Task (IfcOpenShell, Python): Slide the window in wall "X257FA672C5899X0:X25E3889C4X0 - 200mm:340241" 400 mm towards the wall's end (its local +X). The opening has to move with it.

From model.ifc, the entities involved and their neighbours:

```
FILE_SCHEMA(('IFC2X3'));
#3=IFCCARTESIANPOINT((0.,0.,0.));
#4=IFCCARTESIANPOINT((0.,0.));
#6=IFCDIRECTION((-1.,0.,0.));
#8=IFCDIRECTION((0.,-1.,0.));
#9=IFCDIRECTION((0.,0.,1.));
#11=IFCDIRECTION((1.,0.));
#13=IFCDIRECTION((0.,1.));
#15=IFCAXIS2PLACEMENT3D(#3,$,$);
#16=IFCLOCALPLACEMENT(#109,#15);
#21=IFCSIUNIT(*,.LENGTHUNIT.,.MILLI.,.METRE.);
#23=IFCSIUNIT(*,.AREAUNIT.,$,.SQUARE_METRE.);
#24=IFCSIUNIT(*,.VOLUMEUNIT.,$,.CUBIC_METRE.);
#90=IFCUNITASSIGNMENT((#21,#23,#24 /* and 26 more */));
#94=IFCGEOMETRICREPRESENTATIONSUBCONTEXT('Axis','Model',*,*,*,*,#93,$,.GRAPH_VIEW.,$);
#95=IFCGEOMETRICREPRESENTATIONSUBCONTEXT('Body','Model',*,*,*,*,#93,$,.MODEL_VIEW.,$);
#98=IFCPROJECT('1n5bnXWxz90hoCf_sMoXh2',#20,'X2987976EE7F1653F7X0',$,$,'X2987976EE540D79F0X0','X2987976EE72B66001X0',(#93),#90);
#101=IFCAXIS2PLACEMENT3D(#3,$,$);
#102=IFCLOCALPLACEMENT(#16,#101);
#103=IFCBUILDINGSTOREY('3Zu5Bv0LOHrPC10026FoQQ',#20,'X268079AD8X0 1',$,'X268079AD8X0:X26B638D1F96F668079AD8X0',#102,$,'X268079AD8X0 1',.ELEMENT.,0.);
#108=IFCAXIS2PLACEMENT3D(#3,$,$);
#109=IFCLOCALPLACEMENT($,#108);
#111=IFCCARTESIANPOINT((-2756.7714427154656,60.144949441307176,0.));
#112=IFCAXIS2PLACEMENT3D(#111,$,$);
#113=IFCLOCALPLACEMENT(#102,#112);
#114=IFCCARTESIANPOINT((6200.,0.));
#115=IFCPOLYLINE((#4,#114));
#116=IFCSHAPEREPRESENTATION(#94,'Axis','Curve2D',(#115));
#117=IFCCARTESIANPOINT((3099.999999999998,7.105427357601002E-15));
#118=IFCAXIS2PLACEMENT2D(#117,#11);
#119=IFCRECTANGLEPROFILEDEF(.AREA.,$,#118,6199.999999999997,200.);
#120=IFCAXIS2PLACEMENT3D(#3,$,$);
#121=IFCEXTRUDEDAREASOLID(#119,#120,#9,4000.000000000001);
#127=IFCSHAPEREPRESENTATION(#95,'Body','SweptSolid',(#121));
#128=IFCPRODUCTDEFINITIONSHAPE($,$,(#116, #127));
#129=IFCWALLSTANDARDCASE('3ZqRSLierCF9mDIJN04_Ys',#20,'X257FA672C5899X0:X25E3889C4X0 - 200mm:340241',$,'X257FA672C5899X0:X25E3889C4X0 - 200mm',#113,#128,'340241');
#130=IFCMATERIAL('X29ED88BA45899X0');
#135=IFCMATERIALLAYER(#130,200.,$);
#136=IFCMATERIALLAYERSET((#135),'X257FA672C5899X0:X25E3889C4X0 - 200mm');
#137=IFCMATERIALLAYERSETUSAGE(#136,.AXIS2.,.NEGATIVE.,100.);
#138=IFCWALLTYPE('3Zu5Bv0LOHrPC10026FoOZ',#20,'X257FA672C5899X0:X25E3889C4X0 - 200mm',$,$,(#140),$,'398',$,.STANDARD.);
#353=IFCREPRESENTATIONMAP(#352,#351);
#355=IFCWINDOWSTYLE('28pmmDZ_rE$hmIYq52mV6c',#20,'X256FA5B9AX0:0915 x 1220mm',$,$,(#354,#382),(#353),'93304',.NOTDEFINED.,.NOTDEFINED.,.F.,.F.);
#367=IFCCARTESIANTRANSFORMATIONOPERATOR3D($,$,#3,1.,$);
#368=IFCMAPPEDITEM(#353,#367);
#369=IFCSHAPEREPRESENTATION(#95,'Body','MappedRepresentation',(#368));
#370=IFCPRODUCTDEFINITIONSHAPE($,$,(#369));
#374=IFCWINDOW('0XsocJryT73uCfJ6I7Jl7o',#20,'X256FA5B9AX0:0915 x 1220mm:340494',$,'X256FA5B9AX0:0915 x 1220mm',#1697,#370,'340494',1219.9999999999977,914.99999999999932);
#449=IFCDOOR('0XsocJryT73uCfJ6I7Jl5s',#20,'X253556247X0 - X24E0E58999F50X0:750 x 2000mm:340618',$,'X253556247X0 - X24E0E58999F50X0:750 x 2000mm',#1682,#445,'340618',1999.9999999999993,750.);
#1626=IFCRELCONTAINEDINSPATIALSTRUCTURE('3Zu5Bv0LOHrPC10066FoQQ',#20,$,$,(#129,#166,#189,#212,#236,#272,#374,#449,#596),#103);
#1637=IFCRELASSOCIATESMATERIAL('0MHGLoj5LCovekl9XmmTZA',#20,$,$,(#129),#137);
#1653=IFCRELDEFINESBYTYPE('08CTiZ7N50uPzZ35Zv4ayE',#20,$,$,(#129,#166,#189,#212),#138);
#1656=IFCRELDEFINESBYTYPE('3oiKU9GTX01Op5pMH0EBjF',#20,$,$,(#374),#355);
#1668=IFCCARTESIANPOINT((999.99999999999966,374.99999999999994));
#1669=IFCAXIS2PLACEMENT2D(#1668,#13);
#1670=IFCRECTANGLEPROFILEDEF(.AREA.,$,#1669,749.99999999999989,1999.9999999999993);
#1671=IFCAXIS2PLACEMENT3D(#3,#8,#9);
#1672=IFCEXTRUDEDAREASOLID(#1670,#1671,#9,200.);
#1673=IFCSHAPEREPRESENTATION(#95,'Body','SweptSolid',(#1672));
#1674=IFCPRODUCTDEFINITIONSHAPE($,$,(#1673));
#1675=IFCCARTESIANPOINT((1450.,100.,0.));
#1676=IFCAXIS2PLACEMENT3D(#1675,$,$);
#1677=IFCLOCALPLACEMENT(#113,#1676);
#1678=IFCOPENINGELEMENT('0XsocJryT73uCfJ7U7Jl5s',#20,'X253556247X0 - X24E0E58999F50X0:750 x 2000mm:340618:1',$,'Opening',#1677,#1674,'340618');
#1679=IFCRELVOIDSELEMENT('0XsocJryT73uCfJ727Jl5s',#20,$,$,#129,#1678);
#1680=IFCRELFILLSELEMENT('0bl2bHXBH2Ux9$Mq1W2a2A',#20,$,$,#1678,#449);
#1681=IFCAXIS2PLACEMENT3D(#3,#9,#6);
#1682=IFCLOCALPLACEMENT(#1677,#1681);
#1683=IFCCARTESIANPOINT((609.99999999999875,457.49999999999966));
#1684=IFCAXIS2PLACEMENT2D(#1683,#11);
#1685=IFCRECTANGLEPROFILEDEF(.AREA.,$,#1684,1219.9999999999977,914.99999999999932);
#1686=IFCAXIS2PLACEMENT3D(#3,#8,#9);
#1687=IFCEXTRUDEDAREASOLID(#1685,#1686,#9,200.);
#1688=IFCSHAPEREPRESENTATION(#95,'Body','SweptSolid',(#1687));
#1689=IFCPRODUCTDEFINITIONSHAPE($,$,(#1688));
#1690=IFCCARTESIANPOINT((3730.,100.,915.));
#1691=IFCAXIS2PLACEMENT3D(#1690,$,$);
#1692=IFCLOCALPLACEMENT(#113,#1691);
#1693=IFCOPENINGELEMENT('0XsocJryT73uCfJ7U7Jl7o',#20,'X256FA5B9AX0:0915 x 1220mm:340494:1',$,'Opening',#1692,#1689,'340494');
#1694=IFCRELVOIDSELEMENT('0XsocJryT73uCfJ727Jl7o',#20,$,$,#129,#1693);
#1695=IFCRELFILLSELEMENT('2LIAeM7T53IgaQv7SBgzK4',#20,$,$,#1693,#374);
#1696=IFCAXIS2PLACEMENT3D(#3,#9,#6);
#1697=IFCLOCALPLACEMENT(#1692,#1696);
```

```python
import ifcopenshell
import ifcopenshell.api.geometry
import ifcopenshell.util.placement

model = ifcopenshell.open("model.ifc")

window = model.by_guid("0XsocJryT73uCfJ6I7Jl7o")
opening = window.FillsVoids[0].RelatingOpeningElement
wall = opening.VoidsElements[0].RelatingBuildingElement

wall_matrix = ifcopenshell.util.placement.get_local_placement(wall.ObjectPlacement)
shift = wall_matrix[:3, 0] * 400.0
before = ifcopenshell.util.placement.get_local_placement(window.ObjectPlacement)[:3, 3].copy()

# The window is placed relative to its opening, so it follows when the opening moves.
matrix = ifcopenshell.util.placement.get_local_placement(opening.ObjectPlacement)
matrix[:3, 3] += shift
ifcopenshell.api.geometry.edit_object_placement(
    model, product=opening, matrix=matrix, is_si=False, should_transform_children=True
)

after = ifcopenshell.util.placement.get_local_placement(window.ObjectPlacement)[:3, 3]
print("window moved by", (after - before).round(3) + 0.0)

model.write("model_edited.ifc")
```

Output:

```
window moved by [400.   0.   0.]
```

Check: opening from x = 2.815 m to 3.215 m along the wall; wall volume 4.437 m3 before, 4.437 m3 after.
